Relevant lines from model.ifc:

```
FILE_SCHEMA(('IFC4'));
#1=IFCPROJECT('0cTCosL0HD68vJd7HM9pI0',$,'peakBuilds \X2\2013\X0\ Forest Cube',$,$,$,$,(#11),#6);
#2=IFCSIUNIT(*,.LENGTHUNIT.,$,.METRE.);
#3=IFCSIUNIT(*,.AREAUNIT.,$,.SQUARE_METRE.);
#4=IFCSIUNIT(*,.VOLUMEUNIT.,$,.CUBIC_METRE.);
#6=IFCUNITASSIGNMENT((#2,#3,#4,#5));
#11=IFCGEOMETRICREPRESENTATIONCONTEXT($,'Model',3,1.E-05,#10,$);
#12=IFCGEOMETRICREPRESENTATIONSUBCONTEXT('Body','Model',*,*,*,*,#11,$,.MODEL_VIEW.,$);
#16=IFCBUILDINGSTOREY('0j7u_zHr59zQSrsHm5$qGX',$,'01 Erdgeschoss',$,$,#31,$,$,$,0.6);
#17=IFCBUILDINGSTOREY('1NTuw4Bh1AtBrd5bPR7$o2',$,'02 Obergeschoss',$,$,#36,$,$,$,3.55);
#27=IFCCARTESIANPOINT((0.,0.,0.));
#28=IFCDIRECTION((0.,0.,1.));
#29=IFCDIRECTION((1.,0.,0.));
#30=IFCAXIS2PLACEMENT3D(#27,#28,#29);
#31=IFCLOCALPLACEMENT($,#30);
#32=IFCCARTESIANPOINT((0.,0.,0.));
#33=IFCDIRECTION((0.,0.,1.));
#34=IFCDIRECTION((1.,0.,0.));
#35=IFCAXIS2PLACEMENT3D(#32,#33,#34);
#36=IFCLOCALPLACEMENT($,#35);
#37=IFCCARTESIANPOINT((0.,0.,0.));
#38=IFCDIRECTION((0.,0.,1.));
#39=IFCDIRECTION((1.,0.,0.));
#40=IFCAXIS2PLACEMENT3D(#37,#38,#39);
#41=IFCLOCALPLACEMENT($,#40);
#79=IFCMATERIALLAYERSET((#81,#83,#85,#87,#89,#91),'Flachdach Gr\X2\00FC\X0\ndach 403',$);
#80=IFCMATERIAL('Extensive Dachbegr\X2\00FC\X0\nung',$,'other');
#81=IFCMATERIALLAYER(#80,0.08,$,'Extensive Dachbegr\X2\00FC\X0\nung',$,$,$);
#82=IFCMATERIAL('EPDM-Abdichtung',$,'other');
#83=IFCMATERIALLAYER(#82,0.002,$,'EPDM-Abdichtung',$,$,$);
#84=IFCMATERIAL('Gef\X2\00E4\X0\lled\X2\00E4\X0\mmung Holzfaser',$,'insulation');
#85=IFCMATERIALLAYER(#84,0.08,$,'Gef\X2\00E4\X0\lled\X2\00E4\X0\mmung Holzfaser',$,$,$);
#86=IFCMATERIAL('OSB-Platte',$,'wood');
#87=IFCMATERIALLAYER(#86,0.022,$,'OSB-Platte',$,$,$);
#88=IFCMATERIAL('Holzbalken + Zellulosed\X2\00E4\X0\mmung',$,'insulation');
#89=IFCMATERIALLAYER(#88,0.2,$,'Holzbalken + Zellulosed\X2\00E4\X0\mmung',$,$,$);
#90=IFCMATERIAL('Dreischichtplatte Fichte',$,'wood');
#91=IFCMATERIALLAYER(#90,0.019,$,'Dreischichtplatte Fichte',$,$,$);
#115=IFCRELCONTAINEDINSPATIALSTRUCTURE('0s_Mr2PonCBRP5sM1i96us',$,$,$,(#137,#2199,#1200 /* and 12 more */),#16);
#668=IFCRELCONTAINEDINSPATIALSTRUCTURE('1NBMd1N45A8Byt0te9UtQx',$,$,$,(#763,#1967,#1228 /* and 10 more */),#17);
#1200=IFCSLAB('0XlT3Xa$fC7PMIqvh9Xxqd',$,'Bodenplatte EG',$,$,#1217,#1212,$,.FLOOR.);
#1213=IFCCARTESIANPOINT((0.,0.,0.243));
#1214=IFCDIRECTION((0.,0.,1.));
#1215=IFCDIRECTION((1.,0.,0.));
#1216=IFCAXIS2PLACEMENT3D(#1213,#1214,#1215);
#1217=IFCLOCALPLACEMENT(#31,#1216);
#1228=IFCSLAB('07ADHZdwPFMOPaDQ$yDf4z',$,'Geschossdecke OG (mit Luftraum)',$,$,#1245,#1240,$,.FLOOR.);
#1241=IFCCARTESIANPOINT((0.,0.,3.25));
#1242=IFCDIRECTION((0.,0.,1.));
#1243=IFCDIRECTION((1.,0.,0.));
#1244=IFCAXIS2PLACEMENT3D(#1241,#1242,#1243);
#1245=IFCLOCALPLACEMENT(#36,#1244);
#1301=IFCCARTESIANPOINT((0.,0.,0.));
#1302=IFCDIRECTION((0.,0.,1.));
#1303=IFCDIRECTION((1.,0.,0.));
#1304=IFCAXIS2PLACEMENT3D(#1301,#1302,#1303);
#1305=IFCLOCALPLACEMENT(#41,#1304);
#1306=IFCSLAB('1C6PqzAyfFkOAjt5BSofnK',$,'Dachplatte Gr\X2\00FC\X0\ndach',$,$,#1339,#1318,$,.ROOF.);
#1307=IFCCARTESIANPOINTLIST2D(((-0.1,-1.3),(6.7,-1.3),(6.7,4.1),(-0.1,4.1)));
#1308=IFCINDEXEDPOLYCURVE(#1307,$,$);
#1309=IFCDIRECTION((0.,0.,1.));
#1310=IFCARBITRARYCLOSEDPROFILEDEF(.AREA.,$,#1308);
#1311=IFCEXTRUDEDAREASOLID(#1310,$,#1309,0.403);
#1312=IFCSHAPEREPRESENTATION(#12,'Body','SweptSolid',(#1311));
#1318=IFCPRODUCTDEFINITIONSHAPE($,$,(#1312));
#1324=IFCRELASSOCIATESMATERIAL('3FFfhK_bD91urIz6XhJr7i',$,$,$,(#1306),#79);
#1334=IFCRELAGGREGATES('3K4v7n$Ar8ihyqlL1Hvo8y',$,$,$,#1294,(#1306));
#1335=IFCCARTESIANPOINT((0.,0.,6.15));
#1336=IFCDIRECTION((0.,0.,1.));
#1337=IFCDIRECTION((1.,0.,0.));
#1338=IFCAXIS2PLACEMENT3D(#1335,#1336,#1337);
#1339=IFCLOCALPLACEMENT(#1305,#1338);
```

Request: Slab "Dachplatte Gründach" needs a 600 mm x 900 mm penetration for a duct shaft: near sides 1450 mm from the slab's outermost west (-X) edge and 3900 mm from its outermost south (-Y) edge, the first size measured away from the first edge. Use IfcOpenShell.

```python
import numpy as np
import ifcopenshell
import ifcopenshell.api.feature
import ifcopenshell.api.geometry
import ifcopenshell.api.root
import ifcopenshell.geom
import ifcopenshell.util.placement
import ifcopenshell.util.representation
import ifcopenshell.util.shape
import ifcopenshell.util.unit

model = ifcopenshell.open("model.ifc")
unit_scale = ifcopenshell.util.unit.calculate_unit_scale(model)
settings = ifcopenshell.geom.settings()


def volume(element):
    """Net volume in cubic metres, openings subtracted."""
    shape = ifcopenshell.geom.create_shape(settings, element)
    return ifcopenshell.util.shape.get_volume(shape.geometry)


slab = model.by_guid("1C6PqzAyfFkOAjt5BSofnK")
before = volume(slab)

# Extent in the slab's own axes, in metres. The edges named are its -X and -Y sides.
slab_shape = ifcopenshell.geom.create_shape(settings, slab)
vertices = ifcopenshell.util.shape.get_vertices(slab_shape.geometry)
x_min, y_min, bottom = vertices.min(axis=0)
top = vertices[:, 2].max()

opening = ifcopenshell.api.root.create_entity(model, ifc_class="IfcOpeningElement", name="Duct shaft opening", predefined_type="OPENING")
context = ifcopenshell.util.representation.get_context(model, "Model", "Body", "MODEL_VIEW")
width, depth = 0.6, 0.9
outline = [(0.0, 0.0), (width, 0.0), (width, depth), (0.0, depth), (0.0, 0.0)]
# Overshoot both faces by 50 mm so the cut is clean.
shape = ifcopenshell.api.geometry.add_slab_representation(
    model, context=context, depth=top - bottom + 0.1, polyline=outline
)
ifcopenshell.api.geometry.assign_representation(model, product=opening, representation=shape)

matrix = ifcopenshell.util.placement.get_local_placement(slab.ObjectPlacement)
matrix[:, 3] = matrix @ np.append(np.array([x_min + 1.45, y_min + 3.9, bottom - 0.05]) / unit_scale, 1.0)
ifcopenshell.api.geometry.edit_object_placement(model, product=opening, matrix=matrix, is_si=False)
ifcopenshell.api.feature.add_feature(model, feature=opening, element=slab)

after = volume(slab)

print(f"slab volume {before:.3f} -> {after:.3f} m3")

model.write("model_updated.ifc")
```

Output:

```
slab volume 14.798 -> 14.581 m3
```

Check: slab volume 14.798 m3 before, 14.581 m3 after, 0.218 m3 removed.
